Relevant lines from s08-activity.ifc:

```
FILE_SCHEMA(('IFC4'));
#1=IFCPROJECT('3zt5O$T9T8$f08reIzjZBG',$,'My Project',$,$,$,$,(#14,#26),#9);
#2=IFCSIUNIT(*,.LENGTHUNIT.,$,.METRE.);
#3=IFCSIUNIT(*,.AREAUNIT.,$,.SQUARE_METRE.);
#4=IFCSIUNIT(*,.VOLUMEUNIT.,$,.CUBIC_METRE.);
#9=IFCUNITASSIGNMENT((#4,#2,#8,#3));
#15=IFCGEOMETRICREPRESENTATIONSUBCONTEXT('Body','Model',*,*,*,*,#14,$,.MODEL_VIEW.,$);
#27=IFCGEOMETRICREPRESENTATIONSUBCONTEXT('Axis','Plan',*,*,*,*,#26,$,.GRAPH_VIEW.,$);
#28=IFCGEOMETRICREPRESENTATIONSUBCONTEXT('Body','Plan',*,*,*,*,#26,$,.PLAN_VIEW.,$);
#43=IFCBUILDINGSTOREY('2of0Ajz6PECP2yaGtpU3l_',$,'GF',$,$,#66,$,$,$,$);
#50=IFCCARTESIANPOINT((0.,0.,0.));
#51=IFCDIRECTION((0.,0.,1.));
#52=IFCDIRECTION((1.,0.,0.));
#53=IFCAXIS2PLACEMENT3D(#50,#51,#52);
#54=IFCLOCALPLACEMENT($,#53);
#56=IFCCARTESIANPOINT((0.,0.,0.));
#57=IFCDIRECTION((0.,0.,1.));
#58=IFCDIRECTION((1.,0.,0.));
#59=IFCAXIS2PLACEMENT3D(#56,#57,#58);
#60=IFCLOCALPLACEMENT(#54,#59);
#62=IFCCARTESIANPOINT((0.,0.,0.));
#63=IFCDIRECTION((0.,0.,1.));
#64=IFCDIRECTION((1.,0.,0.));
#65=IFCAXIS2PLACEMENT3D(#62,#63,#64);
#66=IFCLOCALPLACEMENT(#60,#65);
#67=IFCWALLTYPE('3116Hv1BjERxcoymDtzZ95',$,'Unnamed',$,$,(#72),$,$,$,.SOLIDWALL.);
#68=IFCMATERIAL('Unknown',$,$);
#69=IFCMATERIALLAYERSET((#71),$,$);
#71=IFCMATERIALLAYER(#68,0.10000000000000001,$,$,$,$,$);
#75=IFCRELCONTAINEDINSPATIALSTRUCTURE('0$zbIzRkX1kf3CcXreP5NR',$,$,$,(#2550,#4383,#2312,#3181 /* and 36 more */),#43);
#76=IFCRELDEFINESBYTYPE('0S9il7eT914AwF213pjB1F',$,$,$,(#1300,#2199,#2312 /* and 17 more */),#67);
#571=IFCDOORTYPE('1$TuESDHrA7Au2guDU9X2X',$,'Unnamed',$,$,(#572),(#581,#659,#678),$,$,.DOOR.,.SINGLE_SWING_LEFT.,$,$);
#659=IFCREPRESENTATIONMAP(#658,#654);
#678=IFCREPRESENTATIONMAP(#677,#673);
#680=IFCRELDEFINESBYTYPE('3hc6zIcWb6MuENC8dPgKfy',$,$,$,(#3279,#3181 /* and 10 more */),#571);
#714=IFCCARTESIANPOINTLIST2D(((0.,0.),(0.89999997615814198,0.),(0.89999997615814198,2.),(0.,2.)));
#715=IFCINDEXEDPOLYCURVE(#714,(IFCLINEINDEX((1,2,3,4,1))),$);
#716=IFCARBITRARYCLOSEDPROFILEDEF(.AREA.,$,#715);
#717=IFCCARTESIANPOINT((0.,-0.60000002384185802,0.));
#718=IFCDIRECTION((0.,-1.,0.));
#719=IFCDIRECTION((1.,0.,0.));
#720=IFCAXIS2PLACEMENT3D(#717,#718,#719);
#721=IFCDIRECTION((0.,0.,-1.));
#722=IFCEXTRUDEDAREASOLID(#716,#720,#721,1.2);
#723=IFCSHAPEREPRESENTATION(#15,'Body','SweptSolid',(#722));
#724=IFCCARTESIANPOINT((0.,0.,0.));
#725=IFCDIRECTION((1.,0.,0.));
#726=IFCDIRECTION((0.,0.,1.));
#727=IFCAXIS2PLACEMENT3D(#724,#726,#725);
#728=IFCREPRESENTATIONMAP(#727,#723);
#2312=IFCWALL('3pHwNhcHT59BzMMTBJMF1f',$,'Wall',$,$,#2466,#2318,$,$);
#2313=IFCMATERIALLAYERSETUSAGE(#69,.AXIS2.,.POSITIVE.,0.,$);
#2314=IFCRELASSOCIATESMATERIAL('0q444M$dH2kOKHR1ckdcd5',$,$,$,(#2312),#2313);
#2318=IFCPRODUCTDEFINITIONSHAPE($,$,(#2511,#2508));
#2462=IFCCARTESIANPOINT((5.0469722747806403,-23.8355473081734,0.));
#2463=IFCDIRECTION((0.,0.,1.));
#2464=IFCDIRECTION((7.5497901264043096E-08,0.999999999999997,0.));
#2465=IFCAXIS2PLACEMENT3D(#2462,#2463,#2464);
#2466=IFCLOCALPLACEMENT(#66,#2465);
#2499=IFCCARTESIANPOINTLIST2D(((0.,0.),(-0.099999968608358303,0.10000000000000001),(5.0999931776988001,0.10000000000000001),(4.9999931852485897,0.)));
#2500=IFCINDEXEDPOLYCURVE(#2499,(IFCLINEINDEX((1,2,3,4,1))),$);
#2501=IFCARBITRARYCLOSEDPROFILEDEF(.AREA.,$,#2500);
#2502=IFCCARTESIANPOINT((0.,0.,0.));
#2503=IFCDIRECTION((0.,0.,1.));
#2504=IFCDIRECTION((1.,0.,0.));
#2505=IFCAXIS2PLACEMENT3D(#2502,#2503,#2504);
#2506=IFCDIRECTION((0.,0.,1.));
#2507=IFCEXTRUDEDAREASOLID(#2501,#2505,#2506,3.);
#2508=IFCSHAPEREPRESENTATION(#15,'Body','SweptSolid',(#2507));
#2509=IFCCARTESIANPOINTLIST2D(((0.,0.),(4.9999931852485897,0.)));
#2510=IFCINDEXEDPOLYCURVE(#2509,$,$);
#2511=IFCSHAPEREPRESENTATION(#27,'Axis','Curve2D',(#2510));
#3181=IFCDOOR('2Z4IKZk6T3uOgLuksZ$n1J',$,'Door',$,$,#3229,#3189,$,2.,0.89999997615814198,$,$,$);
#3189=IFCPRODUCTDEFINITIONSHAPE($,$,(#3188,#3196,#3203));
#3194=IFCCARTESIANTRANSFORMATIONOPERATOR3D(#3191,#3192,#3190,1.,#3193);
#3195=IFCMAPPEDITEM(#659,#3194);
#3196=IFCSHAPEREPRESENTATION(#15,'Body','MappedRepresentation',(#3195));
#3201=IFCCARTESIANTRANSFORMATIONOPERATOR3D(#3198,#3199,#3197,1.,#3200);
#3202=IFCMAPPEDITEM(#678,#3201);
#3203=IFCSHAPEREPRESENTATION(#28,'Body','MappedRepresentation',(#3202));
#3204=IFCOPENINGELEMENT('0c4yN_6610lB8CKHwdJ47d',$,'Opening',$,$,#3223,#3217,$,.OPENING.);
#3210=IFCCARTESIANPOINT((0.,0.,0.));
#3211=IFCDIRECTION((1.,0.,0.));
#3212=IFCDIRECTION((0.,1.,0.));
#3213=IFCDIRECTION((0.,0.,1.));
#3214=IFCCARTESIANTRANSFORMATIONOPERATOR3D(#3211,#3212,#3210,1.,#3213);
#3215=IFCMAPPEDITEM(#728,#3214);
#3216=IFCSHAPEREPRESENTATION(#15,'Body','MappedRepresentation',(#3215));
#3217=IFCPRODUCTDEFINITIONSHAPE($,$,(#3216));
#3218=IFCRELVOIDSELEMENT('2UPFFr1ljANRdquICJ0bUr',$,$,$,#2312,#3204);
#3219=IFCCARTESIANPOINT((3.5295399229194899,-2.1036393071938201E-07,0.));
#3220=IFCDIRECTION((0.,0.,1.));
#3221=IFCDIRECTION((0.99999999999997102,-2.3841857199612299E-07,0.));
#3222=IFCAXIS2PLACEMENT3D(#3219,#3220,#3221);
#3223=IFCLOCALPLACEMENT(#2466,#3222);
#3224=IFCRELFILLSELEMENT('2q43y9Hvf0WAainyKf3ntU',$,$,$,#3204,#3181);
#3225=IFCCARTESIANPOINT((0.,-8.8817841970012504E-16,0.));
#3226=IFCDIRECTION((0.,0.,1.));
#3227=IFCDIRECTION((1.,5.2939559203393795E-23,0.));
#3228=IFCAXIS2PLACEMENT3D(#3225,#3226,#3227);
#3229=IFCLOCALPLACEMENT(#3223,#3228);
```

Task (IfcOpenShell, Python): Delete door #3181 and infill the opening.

```python
import ifcopenshell
import ifcopenshell.api.feature
import ifcopenshell.api.root
import ifcopenshell.geom
import ifcopenshell.util.shape

model = ifcopenshell.open("s08-activity.ifc")
settings = ifcopenshell.geom.settings()


def volume(element):
    """Net volume in cubic metres, openings subtracted."""
    shape = ifcopenshell.geom.create_shape(settings, element)
    return ifcopenshell.util.shape.get_volume(shape.geometry)


door = model.by_guid("2Z4IKZk6T3uOgLuksZ$n1J")
opening = door.FillsVoids[0].RelatingOpeningElement
wall = opening.VoidsElements[0].RelatingBuildingElement
before = volume(wall)

ifcopenshell.api.root.remove_product(model, product=door)
ifcopenshell.api.feature.remove_feature(model, feature=opening)

after = volume(wall)

print(f"wall volume {before:.3f} -> {after:.3f} m3")

model.write("s08-activity_edited.ifc")
```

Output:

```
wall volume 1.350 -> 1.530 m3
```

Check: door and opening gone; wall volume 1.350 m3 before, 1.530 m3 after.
